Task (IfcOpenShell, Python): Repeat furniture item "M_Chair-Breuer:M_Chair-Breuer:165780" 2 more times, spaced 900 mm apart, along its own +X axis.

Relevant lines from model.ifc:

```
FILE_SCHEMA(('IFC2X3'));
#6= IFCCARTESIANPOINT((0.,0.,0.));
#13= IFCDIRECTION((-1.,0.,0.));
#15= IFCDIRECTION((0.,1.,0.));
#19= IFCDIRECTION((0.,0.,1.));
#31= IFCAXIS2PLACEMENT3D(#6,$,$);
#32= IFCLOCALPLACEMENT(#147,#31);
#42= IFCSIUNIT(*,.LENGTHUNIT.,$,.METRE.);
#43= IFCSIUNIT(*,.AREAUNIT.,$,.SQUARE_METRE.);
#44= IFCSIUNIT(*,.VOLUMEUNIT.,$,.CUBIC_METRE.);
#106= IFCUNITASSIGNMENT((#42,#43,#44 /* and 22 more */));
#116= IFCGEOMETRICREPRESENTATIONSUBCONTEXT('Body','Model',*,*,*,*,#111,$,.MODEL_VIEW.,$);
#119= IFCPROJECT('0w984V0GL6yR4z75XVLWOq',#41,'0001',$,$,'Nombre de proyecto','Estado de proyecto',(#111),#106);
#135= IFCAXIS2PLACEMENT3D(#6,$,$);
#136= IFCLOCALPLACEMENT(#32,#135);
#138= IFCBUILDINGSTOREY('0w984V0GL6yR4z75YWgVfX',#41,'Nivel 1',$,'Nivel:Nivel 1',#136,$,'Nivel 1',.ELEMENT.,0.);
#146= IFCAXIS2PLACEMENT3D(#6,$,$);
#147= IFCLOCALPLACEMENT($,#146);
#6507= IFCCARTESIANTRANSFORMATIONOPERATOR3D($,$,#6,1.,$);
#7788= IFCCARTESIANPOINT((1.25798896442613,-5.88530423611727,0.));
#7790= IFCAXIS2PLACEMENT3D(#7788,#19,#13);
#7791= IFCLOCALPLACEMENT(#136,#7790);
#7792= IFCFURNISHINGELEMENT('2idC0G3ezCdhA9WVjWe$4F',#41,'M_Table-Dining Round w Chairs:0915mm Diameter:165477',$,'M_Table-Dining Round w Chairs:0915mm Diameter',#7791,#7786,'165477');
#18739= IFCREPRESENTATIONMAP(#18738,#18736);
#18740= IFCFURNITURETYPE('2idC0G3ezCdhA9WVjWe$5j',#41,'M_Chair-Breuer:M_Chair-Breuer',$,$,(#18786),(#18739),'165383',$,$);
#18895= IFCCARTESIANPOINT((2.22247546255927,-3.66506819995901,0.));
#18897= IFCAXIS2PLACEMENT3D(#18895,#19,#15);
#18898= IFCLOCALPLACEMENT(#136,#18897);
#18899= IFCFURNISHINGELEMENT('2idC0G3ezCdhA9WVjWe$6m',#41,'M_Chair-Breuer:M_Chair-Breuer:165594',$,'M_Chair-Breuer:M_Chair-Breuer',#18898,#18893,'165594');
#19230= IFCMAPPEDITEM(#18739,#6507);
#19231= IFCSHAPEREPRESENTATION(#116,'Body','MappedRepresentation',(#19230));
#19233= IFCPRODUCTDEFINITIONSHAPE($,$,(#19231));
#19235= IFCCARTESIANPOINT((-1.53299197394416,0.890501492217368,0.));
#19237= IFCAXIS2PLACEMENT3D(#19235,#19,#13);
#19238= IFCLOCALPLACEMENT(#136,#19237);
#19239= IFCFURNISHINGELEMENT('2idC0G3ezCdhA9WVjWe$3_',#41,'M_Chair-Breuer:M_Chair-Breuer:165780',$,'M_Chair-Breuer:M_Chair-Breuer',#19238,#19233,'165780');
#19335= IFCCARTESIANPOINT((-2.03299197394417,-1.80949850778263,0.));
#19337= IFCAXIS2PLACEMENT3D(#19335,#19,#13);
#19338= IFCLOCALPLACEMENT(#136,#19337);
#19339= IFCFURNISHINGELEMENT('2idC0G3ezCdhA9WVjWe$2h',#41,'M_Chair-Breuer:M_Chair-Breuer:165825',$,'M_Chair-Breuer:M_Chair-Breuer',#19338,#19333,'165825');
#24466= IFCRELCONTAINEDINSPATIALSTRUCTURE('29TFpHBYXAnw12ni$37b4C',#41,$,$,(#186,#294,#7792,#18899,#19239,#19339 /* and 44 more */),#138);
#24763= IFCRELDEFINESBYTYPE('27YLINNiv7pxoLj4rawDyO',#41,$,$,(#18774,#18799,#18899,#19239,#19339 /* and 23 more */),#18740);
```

```python
import ifcopenshell
import ifcopenshell.api.geometry
import ifcopenshell.api.root
import ifcopenshell.util.element
import ifcopenshell.util.placement

model = ifcopenshell.open("model.ifc")


def reuse_history(source, copy):
    """copy_class also copies each property set's owner history, people and application; keep the originals."""
    for rel in copy.IsDefinedBy:
        if rel.is_a("IfcRelDefinesByProperties") and (history := rel.RelatingPropertyDefinition.OwnerHistory):
            rel.RelatingPropertyDefinition.OwnerHistory = source.OwnerHistory
            ifcopenshell.util.element.remove_deep2(model, history)


source = model.by_guid("2idC0G3ezCdhA9WVjWe$3_")
base = ifcopenshell.util.placement.get_local_placement(source.ObjectPlacement)
step = base[:3, 0] * 0.9

for i in range(1, 3):
    copy = ifcopenshell.api.root.copy_class(model, product=source)
    copy.Representation = ifcopenshell.util.element.copy_deep(
        model, source.Representation, exclude=["IfcGeometricRepresentationContext", "IfcRepresentationMap"]
    )
    copy.Name = "M_Chair-Breuer:M_Chair-Breuer"
    copy.Tag = None
    reuse_history(source, copy)
    matrix = base.copy()
    matrix[:3, 3] += i * step
    print("added at", matrix[:3, 3].round(3) + 0.0)
    ifcopenshell.api.geometry.edit_object_placement(model, product=copy, matrix=matrix, is_si=False)

model.write("model_rev.ifc")
```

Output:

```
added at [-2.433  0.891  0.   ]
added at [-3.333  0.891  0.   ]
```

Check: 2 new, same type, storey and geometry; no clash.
